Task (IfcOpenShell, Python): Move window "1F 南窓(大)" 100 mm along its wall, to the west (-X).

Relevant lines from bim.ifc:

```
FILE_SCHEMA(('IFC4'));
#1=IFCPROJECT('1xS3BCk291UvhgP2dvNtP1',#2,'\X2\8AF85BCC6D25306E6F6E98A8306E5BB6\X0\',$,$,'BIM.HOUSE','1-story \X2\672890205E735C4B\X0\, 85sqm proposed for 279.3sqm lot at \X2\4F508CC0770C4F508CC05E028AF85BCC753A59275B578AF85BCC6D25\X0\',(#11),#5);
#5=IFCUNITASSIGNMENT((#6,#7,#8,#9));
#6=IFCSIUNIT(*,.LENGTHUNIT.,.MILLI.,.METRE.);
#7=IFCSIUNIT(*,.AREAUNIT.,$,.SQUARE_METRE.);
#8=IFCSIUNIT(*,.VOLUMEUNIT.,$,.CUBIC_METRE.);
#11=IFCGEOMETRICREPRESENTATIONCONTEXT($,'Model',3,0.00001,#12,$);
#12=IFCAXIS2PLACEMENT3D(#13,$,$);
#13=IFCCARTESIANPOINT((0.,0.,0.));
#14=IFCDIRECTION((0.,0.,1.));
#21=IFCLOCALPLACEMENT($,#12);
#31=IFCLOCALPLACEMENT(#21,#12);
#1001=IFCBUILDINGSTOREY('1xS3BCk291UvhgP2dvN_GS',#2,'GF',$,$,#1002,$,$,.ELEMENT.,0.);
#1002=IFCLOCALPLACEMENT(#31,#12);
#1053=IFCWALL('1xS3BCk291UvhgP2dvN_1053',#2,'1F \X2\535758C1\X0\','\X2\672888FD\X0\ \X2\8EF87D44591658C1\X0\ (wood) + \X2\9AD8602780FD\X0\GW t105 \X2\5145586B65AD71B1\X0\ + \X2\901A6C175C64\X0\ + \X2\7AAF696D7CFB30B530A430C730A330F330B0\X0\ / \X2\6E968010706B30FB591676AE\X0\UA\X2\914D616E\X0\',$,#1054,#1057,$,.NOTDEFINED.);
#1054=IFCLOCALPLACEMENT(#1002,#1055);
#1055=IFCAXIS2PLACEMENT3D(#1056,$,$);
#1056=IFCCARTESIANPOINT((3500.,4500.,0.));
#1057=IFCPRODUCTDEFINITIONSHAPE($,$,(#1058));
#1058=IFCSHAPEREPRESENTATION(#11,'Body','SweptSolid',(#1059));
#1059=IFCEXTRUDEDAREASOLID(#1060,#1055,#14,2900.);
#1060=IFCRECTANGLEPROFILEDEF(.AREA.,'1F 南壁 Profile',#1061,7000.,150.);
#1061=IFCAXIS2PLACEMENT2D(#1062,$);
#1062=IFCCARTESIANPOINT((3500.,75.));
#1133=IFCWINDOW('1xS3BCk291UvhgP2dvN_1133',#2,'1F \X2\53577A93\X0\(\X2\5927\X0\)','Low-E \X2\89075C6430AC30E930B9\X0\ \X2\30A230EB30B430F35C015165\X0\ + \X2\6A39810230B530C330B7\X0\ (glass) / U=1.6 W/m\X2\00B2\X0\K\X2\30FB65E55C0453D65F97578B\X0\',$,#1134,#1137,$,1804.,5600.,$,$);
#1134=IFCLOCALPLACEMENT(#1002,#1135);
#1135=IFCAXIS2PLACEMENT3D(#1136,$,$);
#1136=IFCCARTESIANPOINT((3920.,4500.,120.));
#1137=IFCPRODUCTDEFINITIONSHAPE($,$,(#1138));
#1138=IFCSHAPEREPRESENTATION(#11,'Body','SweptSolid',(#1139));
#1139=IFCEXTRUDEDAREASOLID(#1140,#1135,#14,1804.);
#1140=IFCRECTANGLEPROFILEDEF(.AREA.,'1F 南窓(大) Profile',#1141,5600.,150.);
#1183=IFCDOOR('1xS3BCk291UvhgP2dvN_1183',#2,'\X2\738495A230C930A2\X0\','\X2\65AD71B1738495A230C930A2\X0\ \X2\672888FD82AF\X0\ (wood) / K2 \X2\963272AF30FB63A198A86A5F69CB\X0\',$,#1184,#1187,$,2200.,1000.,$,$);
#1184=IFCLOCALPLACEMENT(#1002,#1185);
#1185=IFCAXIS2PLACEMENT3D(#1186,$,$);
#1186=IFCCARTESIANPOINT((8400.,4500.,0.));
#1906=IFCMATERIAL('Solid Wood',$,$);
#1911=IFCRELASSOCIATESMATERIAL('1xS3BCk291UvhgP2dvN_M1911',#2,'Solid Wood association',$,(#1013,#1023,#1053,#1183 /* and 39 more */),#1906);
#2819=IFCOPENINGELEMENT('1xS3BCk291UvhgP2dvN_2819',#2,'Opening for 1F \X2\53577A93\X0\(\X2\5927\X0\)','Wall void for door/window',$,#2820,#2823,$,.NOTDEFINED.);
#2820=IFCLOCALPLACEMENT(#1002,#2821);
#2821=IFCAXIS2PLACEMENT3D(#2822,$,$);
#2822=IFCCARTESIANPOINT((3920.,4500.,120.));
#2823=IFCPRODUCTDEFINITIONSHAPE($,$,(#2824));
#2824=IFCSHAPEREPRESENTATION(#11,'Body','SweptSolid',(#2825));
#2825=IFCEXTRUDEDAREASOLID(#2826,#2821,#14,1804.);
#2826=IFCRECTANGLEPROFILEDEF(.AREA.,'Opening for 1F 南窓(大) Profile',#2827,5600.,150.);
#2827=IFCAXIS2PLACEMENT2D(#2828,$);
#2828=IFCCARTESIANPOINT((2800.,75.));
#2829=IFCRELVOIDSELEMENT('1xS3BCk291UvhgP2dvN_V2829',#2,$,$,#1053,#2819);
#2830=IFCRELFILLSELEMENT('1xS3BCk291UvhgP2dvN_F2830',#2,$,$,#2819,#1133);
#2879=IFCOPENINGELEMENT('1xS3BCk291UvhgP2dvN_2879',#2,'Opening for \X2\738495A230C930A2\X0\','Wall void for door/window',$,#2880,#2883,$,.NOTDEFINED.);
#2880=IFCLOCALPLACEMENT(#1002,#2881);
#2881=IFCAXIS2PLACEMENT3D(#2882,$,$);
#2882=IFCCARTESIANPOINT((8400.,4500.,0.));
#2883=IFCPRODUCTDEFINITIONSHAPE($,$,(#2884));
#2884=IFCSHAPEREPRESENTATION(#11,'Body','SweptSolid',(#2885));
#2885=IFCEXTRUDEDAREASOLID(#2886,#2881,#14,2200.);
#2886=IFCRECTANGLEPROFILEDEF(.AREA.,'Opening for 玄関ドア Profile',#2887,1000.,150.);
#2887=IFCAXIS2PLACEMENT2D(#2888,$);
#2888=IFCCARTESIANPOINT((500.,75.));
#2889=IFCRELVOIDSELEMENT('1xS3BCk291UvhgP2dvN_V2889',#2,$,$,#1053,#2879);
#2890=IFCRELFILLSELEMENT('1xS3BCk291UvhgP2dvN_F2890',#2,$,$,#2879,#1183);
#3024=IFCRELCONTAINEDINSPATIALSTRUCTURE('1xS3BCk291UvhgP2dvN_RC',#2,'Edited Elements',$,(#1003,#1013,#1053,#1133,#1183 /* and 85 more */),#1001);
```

```python
import ifcopenshell
import ifcopenshell.api.geometry
import ifcopenshell.util.placement

model = ifcopenshell.open("bim.ifc")

window = model.by_id(1133)
opening = window.FillsVoids[0].RelatingOpeningElement
wall = opening.VoidsElements[0].RelatingBuildingElement

wall_matrix = ifcopenshell.util.placement.get_local_placement(wall.ObjectPlacement)
shift = wall_matrix[:3, 0] * -100.0
before = ifcopenshell.util.placement.get_local_placement(window.ObjectPlacement)[:3, 3].copy()

# The window is not placed relative to its opening, so move both.
for product in (opening, window):
    matrix = ifcopenshell.util.placement.get_local_placement(product.ObjectPlacement)
    matrix[:3, 3] += shift
    ifcopenshell.api.geometry.edit_object_placement(model, product=product, matrix=matrix, is_si=False)

after = ifcopenshell.util.placement.get_local_placement(window.ObjectPlacement)[:3, 3]
print("window moved by", (after - before).round(3) + 0.0)

model.write("bim_v2.ifc")
```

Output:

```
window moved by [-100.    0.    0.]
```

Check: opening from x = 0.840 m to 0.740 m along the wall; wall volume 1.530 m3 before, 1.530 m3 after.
